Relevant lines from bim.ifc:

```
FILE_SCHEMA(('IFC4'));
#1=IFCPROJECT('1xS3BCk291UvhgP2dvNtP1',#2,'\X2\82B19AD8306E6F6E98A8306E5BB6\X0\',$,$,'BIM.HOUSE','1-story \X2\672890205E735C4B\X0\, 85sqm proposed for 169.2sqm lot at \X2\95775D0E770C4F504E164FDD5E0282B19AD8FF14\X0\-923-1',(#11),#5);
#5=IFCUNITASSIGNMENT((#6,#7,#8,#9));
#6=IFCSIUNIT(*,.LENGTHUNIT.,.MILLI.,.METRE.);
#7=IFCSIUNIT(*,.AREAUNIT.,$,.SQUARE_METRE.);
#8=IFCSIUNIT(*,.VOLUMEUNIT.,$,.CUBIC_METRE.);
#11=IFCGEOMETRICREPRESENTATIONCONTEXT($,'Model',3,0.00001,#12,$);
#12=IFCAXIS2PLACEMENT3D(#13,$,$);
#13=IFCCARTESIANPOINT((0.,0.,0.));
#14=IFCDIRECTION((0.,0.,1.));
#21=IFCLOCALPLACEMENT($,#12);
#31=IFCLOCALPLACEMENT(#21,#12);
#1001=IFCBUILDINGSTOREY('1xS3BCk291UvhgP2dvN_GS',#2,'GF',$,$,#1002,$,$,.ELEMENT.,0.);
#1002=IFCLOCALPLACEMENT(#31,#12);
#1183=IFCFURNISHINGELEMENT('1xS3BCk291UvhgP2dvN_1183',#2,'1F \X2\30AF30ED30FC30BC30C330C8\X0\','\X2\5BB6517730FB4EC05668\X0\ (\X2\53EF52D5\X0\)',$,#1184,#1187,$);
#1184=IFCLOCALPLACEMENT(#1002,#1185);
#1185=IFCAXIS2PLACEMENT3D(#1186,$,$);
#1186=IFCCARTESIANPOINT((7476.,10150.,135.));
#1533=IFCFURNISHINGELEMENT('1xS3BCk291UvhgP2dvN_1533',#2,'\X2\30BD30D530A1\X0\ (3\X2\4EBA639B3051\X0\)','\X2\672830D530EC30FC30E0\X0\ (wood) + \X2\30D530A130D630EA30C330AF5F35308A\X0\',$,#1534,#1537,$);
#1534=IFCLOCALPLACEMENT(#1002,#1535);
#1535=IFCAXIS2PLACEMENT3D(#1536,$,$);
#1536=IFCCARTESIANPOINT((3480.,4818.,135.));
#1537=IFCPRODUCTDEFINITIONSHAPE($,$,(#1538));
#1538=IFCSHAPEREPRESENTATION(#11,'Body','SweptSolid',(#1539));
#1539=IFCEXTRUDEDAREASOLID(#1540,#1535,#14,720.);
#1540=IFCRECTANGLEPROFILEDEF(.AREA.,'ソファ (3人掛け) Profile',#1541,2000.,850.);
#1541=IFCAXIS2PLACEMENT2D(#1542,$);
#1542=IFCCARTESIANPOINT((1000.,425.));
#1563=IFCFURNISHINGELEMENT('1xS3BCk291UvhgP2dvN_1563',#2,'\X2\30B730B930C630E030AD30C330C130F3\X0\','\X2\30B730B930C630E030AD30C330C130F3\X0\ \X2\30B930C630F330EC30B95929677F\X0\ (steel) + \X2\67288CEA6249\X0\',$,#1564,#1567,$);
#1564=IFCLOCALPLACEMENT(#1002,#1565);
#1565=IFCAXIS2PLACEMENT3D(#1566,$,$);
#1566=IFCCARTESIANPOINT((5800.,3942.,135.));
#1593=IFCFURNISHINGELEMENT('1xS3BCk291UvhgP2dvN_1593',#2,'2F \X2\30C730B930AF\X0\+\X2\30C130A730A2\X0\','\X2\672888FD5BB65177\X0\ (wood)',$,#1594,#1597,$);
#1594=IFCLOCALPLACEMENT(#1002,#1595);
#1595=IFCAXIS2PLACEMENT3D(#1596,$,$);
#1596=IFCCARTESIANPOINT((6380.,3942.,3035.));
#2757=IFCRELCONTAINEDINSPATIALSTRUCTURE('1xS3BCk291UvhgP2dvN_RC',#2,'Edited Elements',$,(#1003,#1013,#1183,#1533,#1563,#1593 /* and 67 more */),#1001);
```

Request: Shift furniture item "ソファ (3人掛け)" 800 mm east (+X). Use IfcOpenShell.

```python
import ifcopenshell
import ifcopenshell.api.geometry
import ifcopenshell.util.placement
import ifcopenshell.util.unit

model = ifcopenshell.open("bim.ifc")
unit_scale = ifcopenshell.util.unit.calculate_unit_scale(model)

item = model.by_guid("1xS3BCk291UvhgP2dvN_1533")
matrix = ifcopenshell.util.placement.get_local_placement(item.ObjectPlacement)
matrix[0, 3] += 0.8 / unit_scale
ifcopenshell.api.geometry.edit_object_placement(model, product=item, matrix=matrix, is_si=False)

print(ifcopenshell.util.placement.get_local_placement(item.ObjectPlacement).round(3) + 0.0)

model.write("bim_updated.ifc")
```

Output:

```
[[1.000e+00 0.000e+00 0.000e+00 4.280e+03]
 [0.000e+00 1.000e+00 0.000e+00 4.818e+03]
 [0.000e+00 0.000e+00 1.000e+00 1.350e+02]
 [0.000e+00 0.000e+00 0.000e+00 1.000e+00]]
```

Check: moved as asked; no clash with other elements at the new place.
